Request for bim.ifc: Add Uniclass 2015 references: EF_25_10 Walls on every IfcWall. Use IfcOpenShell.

First a look at what the model holds.

```python
import ifcopenshell

model = ifcopenshell.open("bim.ifc")
print(model.schema)
print("classifications:", [c.Name for c in model.by_type("IfcClassification")])
for ifc_class in ("IfcDoor", "IfcRoof", "IfcStair", "IfcWall", "IfcWindow"):
    print(ifc_class, len(model.by_type(ifc_class)))
```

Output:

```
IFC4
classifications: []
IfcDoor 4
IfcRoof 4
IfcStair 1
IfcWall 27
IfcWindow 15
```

```python
import ifcopenshell
import ifcopenshell.api.classification

model = ifcopenshell.open("bim.ifc")

system = ifcopenshell.api.classification.add_classification(model, classification="Uniclass 2015")

codes = {
    "IfcWall": ("EF_25_10", "Walls"),
}
for ifc_class, (code, name) in codes.items():
    products = model.by_type(ifc_class)
    ifcopenshell.api.classification.add_reference(
        model, products=products, classification=system, identification=code, name=name
    )
    print(code, len(products))

model.write("bim_v2.ifc")
```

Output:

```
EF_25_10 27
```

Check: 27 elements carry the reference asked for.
